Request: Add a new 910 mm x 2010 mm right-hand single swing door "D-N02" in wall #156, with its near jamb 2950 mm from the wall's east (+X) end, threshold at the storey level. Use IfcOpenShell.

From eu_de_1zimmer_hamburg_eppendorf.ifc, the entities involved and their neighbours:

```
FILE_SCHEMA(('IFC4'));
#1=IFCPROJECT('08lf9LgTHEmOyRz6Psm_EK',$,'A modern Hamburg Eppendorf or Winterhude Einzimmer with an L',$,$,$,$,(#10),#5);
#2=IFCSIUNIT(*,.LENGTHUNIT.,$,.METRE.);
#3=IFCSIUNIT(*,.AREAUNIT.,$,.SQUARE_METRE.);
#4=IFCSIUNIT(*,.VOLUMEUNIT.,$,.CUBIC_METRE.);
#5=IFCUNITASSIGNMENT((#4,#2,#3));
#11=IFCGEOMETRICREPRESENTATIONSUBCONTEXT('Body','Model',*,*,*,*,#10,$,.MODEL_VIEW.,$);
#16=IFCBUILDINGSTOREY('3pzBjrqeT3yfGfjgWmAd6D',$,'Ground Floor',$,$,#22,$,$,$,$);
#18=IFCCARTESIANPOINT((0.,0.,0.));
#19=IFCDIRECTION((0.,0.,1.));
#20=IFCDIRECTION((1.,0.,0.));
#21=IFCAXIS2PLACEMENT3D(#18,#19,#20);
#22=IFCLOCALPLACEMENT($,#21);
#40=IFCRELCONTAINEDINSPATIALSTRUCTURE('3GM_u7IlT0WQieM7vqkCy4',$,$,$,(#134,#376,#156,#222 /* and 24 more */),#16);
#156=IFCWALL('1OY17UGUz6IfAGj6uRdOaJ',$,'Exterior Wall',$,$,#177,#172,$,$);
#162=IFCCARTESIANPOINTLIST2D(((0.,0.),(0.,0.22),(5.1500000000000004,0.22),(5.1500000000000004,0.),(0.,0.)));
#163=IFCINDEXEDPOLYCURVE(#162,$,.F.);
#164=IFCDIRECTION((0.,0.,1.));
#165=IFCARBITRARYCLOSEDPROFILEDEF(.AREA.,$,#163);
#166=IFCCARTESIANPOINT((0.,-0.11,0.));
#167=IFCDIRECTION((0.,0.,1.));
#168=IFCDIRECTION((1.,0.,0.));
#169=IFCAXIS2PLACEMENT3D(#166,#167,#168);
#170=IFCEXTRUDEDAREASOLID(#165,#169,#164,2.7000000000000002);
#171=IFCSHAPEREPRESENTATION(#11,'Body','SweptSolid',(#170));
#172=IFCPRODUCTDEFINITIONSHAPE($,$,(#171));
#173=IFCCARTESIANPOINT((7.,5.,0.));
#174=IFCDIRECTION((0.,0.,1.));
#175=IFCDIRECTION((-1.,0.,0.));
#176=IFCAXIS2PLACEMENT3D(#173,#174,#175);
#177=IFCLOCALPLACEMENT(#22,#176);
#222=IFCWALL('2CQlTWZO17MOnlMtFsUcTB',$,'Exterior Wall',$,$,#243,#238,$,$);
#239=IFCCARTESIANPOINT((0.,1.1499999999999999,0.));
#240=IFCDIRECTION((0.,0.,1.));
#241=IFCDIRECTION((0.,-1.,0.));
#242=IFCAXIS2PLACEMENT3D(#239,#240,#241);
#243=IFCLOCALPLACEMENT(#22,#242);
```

```python
import numpy as np
import ifcopenshell
import ifcopenshell.api.feature
import ifcopenshell.api.geometry
import ifcopenshell.api.root
import ifcopenshell.api.spatial
import ifcopenshell.geom
import ifcopenshell.util.element
import ifcopenshell.util.placement
import ifcopenshell.util.representation
import ifcopenshell.util.shape
import ifcopenshell.util.unit

model = ifcopenshell.open("eu_de_1zimmer_hamburg_eppendorf.ifc")
unit_scale = ifcopenshell.util.unit.calculate_unit_scale(model)
settings = ifcopenshell.geom.settings()


def volume(element):
    """Net volume in cubic metres, openings subtracted."""
    shape = ifcopenshell.geom.create_shape(settings, element)
    return ifcopenshell.util.shape.get_volume(shape.geometry)


wall = model.by_guid("1OY17UGUz6IfAGj6uRdOaJ")
storey = ifcopenshell.util.element.get_container(wall, ifc_class="IfcBuildingStorey")
context = ifcopenshell.util.representation.get_context(model, "Model", "Body", "MODEL_VIEW")
before = volume(wall)

width, height, from_end, sill = 0.91, 2.01, 2.95, 0.0  # metres

# The wall runs along its own X axis, and the end named is its -X end.
wall_shape = ifcopenshell.geom.create_shape(settings, wall)
x, y, z = ifcopenshell.util.shape.get_vertices(wall_shape.geometry).T
start = x.min() + from_end
face, thickness = float(y.min()), float(y.max() - y.min())
wall_matrix = ifcopenshell.util.placement.get_local_placement(wall.ObjectPlacement)
level = ifcopenshell.util.placement.get_local_placement(storey.ObjectPlacement)[2, 3]


def in_wall(x, y):
    """Placement at x, y metres in the wall's axes, at sill height."""
    matrix = wall_matrix.copy()
    matrix[:, 3] = wall_matrix @ np.array([x / unit_scale, y / unit_scale, 0.0, 1.0])
    matrix[2, 3] = level + sill / unit_scale
    return matrix


# Opening: a box that overshoots both wall faces by 50 mm.
opening = ifcopenshell.api.root.create_entity(model, ifc_class="IfcOpeningElement", predefined_type="OPENING")
box = ifcopenshell.api.geometry.add_wall_representation(
    model, context=context, length=width, height=height, thickness=thickness + 0.1
)
ifcopenshell.api.geometry.assign_representation(model, product=opening, representation=box)
ifcopenshell.api.geometry.edit_object_placement(model, product=opening, matrix=in_wall(start, face - 0.05), is_si=False)
ifcopenshell.api.feature.add_feature(model, feature=opening, element=wall)

door = ifcopenshell.api.root.create_entity(model, ifc_class="IfcDoor", name="D-N02", predefined_type="DOOR")
door.OverallWidth, door.OverallHeight = width / unit_scale, height / unit_scale
door.OperationType = "SINGLE_SWING_RIGHT"
body = ifcopenshell.api.geometry.add_door_representation(
    model,
    context=context,
    overall_width=door.OverallWidth,
    overall_height=door.OverallHeight,
    operation_type="SINGLE_SWING_RIGHT",
    lining_properties={"LiningDepth": thickness / unit_scale, "ThresholdDepth": thickness / unit_scale},
)
ifcopenshell.api.geometry.assign_representation(model, product=door, representation=body)
ifcopenshell.api.spatial.assign_container(model, products=[door], relating_structure=storey)
ifcopenshell.api.feature.add_filling(model, opening=opening, element=door)

# The lining spans the wall, so the door starts at the wall face.
ifcopenshell.api.geometry.edit_object_placement(model, product=door, matrix=in_wall(start, face), is_si=False)

after = volume(wall)

print(f"wall volume {before:.3f} -> {after:.3f} m3")

model.write("eu_de_1zimmer_hamburg_eppendorf_updated.ifc")
```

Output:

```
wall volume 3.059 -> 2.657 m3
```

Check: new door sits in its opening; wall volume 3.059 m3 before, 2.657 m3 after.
